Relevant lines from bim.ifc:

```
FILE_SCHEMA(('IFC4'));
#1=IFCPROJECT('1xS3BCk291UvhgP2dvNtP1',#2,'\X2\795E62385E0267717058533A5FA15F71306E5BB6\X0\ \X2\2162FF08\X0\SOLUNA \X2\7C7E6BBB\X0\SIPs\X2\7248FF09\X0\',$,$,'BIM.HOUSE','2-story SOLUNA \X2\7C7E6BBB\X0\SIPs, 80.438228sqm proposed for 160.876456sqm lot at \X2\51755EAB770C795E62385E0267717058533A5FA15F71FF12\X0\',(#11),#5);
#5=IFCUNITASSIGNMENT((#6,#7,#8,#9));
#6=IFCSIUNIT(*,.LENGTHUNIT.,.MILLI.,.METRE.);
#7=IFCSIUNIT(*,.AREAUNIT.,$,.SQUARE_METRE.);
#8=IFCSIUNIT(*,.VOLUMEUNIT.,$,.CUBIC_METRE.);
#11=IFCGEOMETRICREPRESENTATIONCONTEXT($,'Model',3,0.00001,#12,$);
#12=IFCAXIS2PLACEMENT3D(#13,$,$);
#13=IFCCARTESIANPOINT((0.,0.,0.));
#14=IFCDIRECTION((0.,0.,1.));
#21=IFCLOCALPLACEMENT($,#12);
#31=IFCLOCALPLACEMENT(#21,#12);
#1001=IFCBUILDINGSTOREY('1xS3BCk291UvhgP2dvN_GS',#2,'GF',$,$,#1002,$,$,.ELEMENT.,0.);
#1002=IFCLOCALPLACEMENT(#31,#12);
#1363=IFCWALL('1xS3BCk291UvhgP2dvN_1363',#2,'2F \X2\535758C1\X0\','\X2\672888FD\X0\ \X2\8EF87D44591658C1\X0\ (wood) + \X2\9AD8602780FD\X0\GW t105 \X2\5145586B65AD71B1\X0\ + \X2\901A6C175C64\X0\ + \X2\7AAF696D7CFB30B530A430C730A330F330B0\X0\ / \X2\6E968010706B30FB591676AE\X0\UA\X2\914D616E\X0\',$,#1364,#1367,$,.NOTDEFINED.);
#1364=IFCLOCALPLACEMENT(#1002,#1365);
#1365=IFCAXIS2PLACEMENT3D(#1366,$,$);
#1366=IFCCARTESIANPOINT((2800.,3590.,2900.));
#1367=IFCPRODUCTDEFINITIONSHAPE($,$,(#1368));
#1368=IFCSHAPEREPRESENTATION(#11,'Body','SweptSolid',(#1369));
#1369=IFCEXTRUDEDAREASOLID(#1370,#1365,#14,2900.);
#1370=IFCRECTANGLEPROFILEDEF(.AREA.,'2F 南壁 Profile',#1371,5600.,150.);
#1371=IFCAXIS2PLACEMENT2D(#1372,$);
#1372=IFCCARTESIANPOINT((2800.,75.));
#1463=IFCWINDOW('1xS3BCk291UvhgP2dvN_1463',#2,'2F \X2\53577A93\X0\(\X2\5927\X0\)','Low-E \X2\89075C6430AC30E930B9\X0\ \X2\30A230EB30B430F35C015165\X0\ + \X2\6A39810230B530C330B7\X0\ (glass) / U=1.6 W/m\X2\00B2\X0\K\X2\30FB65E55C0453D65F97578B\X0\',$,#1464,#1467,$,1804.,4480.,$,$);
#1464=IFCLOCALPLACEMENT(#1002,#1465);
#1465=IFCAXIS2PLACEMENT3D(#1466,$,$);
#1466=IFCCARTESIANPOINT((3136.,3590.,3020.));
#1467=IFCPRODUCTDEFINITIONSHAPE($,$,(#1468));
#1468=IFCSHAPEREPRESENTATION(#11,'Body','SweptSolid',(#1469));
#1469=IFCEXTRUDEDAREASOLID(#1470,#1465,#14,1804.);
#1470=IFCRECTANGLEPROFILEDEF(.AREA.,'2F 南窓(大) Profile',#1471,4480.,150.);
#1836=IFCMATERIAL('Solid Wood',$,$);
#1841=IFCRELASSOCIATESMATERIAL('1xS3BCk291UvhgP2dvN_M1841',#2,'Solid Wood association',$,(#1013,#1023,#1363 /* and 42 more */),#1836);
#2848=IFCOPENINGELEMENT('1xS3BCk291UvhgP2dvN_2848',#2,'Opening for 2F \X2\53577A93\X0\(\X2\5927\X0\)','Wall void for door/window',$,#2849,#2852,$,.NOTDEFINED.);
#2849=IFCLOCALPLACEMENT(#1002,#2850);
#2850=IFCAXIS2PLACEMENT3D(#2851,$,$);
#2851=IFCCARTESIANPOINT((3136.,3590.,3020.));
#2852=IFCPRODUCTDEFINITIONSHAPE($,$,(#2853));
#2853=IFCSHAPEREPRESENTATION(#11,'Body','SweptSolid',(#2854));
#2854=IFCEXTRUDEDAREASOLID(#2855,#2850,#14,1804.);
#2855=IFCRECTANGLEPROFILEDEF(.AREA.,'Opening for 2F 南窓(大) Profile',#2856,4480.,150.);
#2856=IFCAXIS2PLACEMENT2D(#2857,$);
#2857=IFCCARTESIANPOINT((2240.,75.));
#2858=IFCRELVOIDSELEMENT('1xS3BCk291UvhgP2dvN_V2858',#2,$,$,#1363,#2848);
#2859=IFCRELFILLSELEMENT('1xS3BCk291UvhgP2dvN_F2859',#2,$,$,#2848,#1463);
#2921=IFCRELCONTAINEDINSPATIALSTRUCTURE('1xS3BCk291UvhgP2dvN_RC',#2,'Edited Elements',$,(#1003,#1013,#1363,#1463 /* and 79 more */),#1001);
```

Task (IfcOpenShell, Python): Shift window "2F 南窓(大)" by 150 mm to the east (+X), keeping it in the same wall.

```python
import ifcopenshell
import ifcopenshell.api.geometry
import ifcopenshell.util.placement

model = ifcopenshell.open("bim.ifc")

window = model.by_guid("1xS3BCk291UvhgP2dvN_1463")
opening = window.FillsVoids[0].RelatingOpeningElement
wall = opening.VoidsElements[0].RelatingBuildingElement

wall_matrix = ifcopenshell.util.placement.get_local_placement(wall.ObjectPlacement)
shift = wall_matrix[:3, 0] * 150.0
before = ifcopenshell.util.placement.get_local_placement(window.ObjectPlacement)[:3, 3].copy()

# The window is not placed relative to its opening, so move both.
for product in (opening, window):
    matrix = ifcopenshell.util.placement.get_local_placement(product.ObjectPlacement)
    matrix[:3, 3] += shift
    ifcopenshell.api.geometry.edit_object_placement(model, product=product, matrix=matrix, is_si=False)

after = ifcopenshell.util.placement.get_local_placement(window.ObjectPlacement)[:3, 3]
print("window moved by", (after - before).round(3) + 0.0)

model.write("bim-out.ifc")
```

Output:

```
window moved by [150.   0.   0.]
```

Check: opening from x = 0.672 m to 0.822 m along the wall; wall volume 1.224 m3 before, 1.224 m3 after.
